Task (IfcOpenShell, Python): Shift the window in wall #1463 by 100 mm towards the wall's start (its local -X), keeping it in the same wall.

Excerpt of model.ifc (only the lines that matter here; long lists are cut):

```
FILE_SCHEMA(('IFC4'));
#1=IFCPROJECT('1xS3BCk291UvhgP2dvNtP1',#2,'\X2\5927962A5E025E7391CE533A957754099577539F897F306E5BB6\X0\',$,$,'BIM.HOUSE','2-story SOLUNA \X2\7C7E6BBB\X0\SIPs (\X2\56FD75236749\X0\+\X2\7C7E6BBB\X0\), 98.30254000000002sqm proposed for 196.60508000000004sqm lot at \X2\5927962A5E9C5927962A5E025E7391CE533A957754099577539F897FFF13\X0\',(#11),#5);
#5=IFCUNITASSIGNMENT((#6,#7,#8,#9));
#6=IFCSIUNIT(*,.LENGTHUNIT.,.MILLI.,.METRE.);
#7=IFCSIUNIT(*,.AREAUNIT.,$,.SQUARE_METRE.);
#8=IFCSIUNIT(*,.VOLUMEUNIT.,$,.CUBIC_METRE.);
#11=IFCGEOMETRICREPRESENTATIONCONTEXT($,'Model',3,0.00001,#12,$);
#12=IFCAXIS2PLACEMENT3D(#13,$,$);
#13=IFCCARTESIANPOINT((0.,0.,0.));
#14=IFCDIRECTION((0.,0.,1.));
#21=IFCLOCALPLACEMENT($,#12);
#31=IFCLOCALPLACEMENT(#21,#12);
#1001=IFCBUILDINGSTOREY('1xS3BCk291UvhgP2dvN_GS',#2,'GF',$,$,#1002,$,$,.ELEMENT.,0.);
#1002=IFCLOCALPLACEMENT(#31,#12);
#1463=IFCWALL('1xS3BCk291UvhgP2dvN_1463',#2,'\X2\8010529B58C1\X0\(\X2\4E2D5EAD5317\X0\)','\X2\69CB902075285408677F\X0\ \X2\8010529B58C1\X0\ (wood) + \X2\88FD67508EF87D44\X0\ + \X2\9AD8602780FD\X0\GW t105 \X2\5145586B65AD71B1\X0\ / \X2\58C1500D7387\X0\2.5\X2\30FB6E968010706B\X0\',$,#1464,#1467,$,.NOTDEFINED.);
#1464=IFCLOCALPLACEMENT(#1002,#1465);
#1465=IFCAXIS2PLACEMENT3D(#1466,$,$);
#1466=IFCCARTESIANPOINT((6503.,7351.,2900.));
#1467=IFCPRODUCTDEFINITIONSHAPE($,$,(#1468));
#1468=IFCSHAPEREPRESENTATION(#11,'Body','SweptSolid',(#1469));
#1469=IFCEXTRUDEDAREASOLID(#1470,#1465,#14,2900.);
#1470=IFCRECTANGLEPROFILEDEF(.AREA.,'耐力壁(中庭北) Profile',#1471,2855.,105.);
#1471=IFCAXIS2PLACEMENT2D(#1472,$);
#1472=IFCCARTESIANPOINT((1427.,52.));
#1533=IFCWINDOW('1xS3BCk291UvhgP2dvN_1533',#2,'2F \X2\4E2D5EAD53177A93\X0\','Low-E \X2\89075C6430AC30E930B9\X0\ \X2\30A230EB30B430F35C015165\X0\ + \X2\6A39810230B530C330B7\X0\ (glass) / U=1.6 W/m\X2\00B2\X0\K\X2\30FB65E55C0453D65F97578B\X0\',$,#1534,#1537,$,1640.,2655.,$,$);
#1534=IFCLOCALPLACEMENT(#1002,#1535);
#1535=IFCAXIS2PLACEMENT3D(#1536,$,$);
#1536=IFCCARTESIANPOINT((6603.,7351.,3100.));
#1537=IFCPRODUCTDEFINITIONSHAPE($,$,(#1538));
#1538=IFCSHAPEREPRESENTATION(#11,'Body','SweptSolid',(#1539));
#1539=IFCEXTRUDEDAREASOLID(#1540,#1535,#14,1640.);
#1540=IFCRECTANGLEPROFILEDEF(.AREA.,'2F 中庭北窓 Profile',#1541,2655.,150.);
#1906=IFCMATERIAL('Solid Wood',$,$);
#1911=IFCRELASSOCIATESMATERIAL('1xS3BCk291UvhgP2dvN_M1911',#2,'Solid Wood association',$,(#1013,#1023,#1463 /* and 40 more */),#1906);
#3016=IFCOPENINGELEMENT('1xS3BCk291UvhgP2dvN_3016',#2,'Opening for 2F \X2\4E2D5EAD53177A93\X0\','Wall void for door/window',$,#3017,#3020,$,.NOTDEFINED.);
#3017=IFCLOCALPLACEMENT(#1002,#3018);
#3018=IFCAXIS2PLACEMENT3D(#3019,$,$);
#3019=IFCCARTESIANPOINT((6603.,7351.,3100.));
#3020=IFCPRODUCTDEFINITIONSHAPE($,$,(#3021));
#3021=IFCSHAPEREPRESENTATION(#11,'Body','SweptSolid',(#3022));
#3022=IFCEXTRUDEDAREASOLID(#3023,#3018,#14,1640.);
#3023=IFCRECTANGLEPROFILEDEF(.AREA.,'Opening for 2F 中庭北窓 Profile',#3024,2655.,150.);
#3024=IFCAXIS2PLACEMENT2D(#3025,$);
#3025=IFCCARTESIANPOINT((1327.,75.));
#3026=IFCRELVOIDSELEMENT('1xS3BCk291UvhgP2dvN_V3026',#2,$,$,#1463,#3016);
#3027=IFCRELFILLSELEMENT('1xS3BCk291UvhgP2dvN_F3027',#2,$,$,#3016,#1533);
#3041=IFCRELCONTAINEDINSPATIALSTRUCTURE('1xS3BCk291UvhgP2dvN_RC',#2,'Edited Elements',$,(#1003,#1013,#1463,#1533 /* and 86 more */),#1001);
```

```python
import ifcopenshell
import ifcopenshell.api.geometry
import ifcopenshell.util.placement

model = ifcopenshell.open("model.ifc")

window = model.by_id(1533)
opening = window.FillsVoids[0].RelatingOpeningElement
wall = opening.VoidsElements[0].RelatingBuildingElement

wall_matrix = ifcopenshell.util.placement.get_local_placement(wall.ObjectPlacement)
shift = wall_matrix[:3, 0] * -100.0
before = ifcopenshell.util.placement.get_local_placement(window.ObjectPlacement)[:3, 3].copy()

# The window is not placed relative to its opening, so move both.
for product in (opening, window):
    matrix = ifcopenshell.util.placement.get_local_placement(product.ObjectPlacement)
    matrix[:3, 3] += shift
    ifcopenshell.api.geometry.edit_object_placement(model, product=product, matrix=matrix, is_si=False)

after = ifcopenshell.util.placement.get_local_placement(window.ObjectPlacement)[:3, 3]
print("window moved by", (after - before).round(3) + 0.0)

model.write("model-out.ifc")
```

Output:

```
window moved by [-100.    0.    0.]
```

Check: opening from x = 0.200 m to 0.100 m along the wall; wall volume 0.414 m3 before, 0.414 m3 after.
